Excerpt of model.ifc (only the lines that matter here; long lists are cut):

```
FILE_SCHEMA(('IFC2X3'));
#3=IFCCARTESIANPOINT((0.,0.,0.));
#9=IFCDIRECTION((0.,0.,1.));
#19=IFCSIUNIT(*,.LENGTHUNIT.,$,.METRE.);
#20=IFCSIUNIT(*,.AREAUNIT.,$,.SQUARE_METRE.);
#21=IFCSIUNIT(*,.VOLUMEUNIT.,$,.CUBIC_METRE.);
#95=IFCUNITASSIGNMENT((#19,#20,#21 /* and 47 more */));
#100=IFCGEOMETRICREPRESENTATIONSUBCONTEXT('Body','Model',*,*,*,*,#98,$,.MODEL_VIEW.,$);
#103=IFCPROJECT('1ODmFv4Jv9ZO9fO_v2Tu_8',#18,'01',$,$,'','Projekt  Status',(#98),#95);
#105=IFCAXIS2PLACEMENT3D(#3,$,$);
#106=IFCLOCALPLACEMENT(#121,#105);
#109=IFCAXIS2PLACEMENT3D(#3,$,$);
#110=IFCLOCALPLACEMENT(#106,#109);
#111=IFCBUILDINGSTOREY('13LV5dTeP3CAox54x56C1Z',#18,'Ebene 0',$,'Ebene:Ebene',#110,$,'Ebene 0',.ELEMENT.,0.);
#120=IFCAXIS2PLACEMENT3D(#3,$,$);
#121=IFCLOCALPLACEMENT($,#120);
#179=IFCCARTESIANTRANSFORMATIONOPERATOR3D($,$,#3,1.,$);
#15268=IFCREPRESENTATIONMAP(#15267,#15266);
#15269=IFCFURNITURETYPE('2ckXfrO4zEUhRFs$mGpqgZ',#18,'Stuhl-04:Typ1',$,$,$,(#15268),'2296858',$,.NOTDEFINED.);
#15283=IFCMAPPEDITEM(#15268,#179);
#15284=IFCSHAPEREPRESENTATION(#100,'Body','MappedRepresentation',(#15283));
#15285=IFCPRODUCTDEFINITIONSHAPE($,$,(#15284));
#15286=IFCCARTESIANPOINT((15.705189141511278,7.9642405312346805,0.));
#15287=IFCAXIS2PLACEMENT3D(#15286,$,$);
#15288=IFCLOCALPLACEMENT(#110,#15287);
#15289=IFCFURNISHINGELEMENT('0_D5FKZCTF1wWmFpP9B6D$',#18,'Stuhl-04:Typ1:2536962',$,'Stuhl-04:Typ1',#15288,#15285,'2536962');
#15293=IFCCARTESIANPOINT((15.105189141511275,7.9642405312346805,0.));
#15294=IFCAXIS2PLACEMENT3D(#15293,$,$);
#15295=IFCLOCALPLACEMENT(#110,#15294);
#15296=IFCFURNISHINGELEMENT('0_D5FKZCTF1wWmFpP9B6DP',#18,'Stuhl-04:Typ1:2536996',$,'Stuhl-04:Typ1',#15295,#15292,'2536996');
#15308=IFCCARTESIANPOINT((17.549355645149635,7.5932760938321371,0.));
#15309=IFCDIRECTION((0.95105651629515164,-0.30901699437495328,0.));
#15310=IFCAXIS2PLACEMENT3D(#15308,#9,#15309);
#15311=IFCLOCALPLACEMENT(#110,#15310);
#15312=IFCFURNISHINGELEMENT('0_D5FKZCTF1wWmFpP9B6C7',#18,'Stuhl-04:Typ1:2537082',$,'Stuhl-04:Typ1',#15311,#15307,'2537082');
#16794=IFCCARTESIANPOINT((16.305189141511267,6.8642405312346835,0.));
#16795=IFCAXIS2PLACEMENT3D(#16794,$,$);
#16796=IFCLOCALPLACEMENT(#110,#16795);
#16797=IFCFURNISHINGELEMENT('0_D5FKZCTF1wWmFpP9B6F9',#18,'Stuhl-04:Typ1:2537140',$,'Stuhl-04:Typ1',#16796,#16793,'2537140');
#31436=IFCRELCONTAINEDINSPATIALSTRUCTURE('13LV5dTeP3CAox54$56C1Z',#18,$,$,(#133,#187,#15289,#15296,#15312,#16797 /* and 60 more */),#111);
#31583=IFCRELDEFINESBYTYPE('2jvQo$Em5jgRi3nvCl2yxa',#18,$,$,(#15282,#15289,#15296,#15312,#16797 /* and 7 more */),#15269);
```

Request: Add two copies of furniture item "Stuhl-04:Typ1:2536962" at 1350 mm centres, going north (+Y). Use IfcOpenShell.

```python
import numpy as np
import ifcopenshell
import ifcopenshell.api.geometry
import ifcopenshell.api.root
import ifcopenshell.util.element
import ifcopenshell.util.placement
import ifcopenshell.util.unit

model = ifcopenshell.open("model.ifc")
unit_scale = ifcopenshell.util.unit.calculate_unit_scale(model)

source = model.by_id(15289)
base = ifcopenshell.util.placement.get_local_placement(source.ObjectPlacement)
step = np.array([0.0, 1.0, 0.0]) * 1.35 / unit_scale

for i in range(1, 3):
    copy = ifcopenshell.api.root.copy_class(model, product=source)
    copy.Representation = ifcopenshell.util.element.copy_deep(
        model, source.Representation, exclude=["IfcGeometricRepresentationContext", "IfcRepresentationMap"]
    )
    copy.Name = "Stuhl-04:Typ1"
    copy.Tag = None
    matrix = base.copy()
    matrix[:3, 3] += i * step
    print("added at", matrix[:3, 3].round(3) + 0.0)
    ifcopenshell.api.geometry.edit_object_placement(model, product=copy, matrix=matrix, is_si=False)

model.write("model_v2.ifc")
```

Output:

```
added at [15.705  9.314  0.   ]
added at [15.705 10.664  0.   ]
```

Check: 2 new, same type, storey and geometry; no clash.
